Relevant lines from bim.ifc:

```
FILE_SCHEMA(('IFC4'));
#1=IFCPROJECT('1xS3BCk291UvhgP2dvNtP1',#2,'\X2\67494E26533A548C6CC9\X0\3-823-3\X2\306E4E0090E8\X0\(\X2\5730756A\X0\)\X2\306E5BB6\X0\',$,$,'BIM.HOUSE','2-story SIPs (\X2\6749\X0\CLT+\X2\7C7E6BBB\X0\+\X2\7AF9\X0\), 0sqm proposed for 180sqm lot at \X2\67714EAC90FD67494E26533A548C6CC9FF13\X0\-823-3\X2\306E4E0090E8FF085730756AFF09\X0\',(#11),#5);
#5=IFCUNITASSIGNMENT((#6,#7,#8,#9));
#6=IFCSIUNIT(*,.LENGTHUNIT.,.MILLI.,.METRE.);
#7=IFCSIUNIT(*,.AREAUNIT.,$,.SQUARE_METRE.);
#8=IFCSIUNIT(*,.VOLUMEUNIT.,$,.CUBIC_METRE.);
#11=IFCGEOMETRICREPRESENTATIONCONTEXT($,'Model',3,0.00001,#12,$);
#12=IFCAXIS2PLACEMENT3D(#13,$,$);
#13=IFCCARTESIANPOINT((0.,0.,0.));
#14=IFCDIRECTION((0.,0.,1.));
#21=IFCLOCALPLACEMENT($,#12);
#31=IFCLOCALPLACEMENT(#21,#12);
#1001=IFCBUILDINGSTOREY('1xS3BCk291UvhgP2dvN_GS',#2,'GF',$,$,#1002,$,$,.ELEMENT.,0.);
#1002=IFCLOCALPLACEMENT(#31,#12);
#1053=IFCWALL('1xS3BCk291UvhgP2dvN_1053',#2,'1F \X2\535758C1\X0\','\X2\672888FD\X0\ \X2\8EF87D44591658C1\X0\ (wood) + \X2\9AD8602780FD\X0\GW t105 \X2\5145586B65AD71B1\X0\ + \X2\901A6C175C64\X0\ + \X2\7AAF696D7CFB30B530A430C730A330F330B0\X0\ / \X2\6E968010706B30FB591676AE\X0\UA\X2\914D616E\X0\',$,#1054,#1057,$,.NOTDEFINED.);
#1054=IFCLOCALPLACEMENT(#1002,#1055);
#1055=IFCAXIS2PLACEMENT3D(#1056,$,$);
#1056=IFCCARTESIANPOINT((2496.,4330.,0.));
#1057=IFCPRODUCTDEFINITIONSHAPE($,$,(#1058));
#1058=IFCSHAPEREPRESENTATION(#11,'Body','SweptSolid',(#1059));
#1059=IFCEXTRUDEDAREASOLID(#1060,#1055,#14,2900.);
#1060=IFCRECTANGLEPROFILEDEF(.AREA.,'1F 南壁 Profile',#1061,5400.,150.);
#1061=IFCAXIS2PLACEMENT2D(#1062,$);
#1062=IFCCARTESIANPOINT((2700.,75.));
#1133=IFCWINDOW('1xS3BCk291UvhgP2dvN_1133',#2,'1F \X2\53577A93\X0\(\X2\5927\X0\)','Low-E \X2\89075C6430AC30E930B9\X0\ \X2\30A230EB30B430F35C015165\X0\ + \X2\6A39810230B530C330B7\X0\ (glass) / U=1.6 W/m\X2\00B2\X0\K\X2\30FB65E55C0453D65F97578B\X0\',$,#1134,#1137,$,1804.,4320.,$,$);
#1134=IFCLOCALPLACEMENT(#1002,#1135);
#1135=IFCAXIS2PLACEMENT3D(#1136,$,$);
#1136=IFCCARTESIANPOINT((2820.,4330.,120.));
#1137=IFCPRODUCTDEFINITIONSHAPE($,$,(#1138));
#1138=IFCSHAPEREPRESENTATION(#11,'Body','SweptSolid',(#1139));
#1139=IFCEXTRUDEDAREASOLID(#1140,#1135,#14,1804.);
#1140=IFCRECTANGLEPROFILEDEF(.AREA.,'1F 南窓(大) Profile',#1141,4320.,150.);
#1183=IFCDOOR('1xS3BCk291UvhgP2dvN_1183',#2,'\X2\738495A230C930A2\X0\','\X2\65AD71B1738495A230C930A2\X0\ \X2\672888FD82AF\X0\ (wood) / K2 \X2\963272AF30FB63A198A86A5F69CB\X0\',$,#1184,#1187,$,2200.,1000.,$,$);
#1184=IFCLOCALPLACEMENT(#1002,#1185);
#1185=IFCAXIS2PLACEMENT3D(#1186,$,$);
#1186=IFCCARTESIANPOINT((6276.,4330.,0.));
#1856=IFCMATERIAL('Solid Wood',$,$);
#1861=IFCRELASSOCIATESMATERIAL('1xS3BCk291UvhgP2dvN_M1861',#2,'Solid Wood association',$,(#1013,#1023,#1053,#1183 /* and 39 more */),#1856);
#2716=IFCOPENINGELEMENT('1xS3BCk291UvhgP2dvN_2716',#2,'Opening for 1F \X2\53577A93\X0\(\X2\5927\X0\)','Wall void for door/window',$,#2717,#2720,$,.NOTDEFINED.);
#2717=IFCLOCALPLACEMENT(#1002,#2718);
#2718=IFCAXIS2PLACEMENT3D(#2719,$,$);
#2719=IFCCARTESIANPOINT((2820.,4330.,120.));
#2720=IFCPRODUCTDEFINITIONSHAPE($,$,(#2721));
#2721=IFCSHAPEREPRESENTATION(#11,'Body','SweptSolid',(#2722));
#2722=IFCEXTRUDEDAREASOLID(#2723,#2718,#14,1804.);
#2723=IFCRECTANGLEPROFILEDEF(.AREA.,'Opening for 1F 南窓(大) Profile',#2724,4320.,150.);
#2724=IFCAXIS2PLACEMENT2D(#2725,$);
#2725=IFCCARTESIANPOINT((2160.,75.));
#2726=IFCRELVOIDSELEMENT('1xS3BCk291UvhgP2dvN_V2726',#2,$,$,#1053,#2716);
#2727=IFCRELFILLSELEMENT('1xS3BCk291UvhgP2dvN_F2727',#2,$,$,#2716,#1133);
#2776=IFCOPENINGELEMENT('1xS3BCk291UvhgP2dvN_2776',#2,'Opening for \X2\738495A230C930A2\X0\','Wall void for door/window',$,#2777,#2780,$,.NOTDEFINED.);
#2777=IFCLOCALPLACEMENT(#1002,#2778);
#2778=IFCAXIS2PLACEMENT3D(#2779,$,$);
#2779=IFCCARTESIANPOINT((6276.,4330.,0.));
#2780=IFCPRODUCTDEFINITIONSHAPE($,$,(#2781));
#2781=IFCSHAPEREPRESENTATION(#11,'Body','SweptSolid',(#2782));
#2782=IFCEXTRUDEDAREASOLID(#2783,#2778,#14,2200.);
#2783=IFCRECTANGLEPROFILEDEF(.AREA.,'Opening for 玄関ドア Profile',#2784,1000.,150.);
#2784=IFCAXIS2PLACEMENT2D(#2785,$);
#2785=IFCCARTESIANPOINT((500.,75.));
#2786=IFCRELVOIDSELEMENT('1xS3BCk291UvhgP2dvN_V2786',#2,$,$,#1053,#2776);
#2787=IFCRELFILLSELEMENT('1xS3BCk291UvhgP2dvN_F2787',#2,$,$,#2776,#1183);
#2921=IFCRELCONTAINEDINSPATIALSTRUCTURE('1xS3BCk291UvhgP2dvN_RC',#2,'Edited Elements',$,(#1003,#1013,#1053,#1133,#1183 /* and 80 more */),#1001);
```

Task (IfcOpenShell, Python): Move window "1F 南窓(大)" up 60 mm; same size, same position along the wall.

```python
import numpy as np
import ifcopenshell
import ifcopenshell.api.geometry
import ifcopenshell.util.placement
import ifcopenshell.util.unit

model = ifcopenshell.open("bim.ifc")
unit_scale = ifcopenshell.util.unit.calculate_unit_scale(model)

window = model.by_guid("1xS3BCk291UvhgP2dvN_1133")
opening = window.FillsVoids[0].RelatingOpeningElement
dz = 0.06 / unit_scale

shift = np.array([0.0, 0.0, dz])
# The window is not placed relative to its opening, so move both.
for product in (opening, window):
    matrix = ifcopenshell.util.placement.get_local_placement(product.ObjectPlacement)
    matrix[:3, 3] += shift
    ifcopenshell.api.geometry.edit_object_placement(model, product=product, matrix=matrix, is_si=False)

print(f"moved by {dz * unit_scale:+.3f} m")

model.write("bim_v2.ifc")
```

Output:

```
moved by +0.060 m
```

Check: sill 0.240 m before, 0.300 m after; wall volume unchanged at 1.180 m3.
